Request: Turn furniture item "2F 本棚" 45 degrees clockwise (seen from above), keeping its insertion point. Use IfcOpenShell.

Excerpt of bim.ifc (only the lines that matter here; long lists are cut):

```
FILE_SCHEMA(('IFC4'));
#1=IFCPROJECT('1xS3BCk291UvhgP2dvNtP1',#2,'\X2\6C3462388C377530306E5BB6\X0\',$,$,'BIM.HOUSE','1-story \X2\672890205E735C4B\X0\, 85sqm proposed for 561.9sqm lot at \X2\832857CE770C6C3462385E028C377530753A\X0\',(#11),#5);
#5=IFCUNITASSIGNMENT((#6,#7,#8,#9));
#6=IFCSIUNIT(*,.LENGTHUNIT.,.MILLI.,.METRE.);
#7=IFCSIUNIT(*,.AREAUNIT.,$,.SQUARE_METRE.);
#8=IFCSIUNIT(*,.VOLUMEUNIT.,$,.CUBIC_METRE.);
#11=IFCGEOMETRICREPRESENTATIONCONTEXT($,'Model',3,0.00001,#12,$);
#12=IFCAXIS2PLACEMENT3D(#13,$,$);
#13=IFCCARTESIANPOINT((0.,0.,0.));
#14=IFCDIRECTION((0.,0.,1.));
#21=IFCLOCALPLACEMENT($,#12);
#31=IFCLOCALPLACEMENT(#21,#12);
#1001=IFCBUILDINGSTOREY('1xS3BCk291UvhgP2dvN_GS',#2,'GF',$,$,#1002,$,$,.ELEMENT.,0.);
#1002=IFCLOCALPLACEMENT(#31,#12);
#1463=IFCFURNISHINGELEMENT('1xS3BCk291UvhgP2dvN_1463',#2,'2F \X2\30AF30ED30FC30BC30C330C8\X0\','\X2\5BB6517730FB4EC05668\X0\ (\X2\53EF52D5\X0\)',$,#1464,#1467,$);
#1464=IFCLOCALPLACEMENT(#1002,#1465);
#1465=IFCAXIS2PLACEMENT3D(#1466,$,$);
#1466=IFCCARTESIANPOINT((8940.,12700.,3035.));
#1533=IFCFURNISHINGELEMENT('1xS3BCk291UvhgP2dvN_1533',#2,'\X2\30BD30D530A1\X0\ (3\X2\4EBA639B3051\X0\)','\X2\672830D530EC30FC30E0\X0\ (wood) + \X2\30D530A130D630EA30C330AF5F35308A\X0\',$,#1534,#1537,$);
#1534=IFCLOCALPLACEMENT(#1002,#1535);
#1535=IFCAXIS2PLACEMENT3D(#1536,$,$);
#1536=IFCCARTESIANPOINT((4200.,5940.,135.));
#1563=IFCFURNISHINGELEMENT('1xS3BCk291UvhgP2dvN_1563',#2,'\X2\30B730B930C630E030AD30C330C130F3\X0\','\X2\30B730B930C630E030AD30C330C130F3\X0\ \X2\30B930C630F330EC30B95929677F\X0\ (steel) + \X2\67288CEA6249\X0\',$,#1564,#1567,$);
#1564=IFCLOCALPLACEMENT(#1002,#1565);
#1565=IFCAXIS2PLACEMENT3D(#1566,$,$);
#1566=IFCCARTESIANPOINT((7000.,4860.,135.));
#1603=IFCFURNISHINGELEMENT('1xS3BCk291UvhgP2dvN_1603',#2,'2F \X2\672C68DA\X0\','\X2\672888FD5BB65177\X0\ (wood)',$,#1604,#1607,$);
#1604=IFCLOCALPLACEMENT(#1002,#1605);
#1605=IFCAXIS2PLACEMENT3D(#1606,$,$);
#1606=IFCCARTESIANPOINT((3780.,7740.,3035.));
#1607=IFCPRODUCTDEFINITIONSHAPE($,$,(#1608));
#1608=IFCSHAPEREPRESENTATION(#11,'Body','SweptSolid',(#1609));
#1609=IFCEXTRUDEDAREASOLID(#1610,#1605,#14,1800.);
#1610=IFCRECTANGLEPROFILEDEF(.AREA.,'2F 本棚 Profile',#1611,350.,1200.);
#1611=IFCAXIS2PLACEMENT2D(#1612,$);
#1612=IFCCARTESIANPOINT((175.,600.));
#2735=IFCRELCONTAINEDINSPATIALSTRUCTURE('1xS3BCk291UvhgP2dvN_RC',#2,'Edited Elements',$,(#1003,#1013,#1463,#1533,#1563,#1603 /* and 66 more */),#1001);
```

```python
import ifcopenshell
import ifcopenshell.api.geometry
import ifcopenshell.util.placement

model = ifcopenshell.open("bim.ifc")

item = model.by_guid("1xS3BCk291UvhgP2dvN_1603")
matrix = ifcopenshell.util.placement.get_local_placement(item.ObjectPlacement)
matrix = matrix @ ifcopenshell.util.placement.rotation(-45, "Z")
ifcopenshell.api.geometry.edit_object_placement(model, product=item, matrix=matrix, is_si=False)

print(ifcopenshell.util.placement.get_local_placement(item.ObjectPlacement).round(3) + 0.0)

model.write("bim-out.ifc")
```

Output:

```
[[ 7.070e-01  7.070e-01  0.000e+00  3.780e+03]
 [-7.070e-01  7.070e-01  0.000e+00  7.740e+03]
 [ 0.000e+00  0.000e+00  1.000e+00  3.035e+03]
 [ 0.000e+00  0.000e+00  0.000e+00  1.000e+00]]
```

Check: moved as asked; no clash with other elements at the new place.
